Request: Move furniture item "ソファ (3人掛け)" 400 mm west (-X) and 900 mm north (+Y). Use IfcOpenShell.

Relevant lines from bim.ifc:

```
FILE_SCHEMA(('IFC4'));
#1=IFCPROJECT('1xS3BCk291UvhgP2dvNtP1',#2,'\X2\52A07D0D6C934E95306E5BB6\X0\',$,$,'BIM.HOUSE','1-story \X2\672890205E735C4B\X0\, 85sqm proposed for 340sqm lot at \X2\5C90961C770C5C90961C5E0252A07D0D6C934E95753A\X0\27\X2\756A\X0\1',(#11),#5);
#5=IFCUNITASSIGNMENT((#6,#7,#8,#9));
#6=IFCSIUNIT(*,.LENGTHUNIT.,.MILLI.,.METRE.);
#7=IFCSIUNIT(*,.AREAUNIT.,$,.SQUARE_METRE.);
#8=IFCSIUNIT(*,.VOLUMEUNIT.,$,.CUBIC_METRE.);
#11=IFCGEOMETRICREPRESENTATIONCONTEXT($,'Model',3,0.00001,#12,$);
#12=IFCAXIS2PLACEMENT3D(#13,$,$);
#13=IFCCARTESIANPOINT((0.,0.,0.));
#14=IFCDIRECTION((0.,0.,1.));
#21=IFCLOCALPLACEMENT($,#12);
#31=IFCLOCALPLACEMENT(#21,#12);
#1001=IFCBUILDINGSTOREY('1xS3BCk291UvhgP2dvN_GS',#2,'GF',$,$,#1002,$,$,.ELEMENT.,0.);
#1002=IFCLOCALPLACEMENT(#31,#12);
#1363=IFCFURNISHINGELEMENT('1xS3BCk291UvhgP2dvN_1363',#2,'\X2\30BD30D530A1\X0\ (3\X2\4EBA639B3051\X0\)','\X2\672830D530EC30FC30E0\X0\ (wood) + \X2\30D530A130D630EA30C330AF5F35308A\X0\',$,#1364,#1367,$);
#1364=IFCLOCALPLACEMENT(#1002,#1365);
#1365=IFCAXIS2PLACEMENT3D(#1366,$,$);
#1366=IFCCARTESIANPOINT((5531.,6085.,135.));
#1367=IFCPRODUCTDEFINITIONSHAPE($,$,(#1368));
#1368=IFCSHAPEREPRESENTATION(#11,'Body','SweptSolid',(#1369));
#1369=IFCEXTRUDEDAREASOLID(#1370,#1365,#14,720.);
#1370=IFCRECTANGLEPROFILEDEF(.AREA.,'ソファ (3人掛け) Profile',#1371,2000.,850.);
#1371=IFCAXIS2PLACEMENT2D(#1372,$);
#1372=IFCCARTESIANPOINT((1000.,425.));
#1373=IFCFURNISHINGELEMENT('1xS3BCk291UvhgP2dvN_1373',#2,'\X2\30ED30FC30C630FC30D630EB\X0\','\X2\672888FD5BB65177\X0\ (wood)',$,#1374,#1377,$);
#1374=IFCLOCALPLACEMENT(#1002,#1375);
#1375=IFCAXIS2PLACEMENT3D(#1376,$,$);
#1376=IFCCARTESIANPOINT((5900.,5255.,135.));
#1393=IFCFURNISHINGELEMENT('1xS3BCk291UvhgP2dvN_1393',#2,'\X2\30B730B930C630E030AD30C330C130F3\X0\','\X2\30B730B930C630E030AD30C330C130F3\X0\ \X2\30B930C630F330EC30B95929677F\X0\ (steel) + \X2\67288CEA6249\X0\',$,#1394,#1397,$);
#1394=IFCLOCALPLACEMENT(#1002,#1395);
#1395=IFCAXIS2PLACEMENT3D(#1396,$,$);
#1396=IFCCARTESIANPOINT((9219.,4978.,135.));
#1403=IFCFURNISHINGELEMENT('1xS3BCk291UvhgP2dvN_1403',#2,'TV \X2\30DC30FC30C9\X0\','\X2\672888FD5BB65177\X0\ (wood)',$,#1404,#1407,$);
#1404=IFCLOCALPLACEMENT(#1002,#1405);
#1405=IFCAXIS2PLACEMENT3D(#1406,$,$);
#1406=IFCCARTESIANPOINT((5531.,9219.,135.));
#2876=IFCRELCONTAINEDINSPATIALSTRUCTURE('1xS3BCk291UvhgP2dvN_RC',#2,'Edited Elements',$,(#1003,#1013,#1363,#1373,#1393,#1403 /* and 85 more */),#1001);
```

```python
import ifcopenshell
import ifcopenshell.api.geometry
import ifcopenshell.util.placement

model = ifcopenshell.open("bim.ifc")

item = model.by_id(1363)
matrix = ifcopenshell.util.placement.get_local_placement(item.ObjectPlacement)
matrix[0, 3] -= 400.0
matrix[1, 3] += 900.0
ifcopenshell.api.geometry.edit_object_placement(model, product=item, matrix=matrix, is_si=False)

print(ifcopenshell.util.placement.get_local_placement(item.ObjectPlacement).round(3) + 0.0)

model.write("bim-out.ifc")
```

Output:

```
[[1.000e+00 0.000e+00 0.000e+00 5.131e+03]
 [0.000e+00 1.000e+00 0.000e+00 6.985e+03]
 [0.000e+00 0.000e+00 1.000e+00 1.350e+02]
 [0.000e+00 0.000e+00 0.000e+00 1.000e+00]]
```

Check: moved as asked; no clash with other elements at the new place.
